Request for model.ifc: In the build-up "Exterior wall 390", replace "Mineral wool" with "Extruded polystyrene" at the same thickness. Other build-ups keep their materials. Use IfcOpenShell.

First a look at what the model holds.

```python
import ifcopenshell
import ifcopenshell.util.element

model = ifcopenshell.open("model.ifc")
print(model.schema)
for layer_set in model.by_type("IfcMaterialLayerSet"):
    if layer_set.LayerSetName == "Exterior wall 390":
        for layer in layer_set.MaterialLayers:
            print(layer.id(), layer.Material and layer.Material.Name, layer.LayerThickness, sep=" | ")
        print(len(ifcopenshell.util.element.get_elements_by_material(model, layer_set)), "elements and types use it")
print(sorted(m.Name for m in model.by_type("IfcMaterial") if m.Name)[:60])
```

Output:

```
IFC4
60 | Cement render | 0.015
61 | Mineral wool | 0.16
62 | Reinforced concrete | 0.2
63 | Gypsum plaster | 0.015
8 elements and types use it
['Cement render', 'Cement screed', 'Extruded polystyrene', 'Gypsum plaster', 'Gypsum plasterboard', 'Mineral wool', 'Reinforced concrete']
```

```python
import ifcopenshell
import ifcopenshell.api.material

model = ifcopenshell.open("model.ifc")

layer_set = next(s for s in model.by_type("IfcMaterialLayerSet") if s.LayerSetName == "Exterior wall 390")
layer = next(l for l in layer_set.MaterialLayers if l.Material and l.Material.Name == "Mineral wool")
material = next(m for m in model.by_type("IfcMaterial") if m.Name == "Extruded polystyrene")

# Point this one layer at the other material; renaming the old one would change it everywhere.
ifcopenshell.api.material.edit_layer(model, layer=layer, attributes={"Name": material.Name}, material=material)

print([l.Material.Name if l.Material else None for l in layer_set.MaterialLayers])

model.write("model-out.ifc")
```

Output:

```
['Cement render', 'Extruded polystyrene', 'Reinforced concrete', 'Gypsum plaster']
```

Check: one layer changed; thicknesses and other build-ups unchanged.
